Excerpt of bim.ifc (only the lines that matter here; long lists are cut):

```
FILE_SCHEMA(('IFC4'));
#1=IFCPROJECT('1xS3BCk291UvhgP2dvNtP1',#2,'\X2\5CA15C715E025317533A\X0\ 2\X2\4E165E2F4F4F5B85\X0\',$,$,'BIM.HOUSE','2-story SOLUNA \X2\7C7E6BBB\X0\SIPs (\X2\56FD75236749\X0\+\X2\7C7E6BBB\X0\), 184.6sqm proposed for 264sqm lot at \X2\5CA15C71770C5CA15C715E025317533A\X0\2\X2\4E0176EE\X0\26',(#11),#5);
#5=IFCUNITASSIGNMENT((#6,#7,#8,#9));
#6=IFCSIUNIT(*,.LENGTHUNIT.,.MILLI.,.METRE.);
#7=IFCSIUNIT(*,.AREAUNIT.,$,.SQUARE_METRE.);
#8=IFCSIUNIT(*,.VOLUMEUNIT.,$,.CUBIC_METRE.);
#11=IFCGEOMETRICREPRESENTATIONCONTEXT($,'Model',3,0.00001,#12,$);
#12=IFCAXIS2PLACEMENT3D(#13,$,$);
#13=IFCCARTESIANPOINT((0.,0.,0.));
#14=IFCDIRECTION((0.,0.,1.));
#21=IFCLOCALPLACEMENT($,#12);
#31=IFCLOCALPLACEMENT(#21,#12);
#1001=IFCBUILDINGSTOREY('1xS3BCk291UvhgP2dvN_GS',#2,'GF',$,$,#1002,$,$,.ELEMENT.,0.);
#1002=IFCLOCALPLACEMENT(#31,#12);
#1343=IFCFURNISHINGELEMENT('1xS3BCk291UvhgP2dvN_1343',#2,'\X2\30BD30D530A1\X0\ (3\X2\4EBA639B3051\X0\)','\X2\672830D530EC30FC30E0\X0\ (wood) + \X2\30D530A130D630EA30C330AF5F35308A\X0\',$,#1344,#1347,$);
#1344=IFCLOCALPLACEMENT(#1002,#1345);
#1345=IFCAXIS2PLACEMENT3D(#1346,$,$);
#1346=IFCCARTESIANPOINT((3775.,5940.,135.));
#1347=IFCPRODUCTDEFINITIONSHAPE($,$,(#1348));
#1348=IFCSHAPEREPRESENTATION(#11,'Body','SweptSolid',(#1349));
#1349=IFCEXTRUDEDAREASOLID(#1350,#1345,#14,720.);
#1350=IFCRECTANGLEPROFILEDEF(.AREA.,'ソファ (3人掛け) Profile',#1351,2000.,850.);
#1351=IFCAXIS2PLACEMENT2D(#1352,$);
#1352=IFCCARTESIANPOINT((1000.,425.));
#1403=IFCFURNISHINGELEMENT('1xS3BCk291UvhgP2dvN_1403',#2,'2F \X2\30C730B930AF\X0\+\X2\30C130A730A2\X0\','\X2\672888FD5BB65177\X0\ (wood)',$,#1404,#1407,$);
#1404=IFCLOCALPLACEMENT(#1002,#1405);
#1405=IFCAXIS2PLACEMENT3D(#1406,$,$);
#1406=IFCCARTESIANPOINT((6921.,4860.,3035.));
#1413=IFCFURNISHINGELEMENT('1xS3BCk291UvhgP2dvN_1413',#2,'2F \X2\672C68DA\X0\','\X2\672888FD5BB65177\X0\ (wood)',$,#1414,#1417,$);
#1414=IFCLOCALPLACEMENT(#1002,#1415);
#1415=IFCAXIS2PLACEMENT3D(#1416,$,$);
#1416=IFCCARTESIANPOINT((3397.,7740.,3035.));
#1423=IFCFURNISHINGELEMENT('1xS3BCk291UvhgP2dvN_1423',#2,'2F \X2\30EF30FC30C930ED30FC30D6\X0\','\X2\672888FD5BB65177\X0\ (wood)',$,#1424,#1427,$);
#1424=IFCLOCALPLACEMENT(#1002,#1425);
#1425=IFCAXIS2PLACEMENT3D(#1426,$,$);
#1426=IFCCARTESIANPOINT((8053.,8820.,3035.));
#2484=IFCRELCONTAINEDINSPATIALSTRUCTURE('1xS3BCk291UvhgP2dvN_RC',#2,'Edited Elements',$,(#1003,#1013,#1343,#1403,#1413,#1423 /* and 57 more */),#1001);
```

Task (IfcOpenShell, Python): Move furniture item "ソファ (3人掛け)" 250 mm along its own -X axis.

```python
import ifcopenshell
import ifcopenshell.api.geometry
import ifcopenshell.util.placement

model = ifcopenshell.open("bim.ifc")

item = model.by_id(1343)
matrix = ifcopenshell.util.placement.get_local_placement(item.ObjectPlacement)
matrix[:3, 3] -= matrix[:3, 0] * 250.0
ifcopenshell.api.geometry.edit_object_placement(model, product=item, matrix=matrix, is_si=False)

print(ifcopenshell.util.placement.get_local_placement(item.ObjectPlacement).round(3) + 0.0)

model.write("bim_edited.ifc")
```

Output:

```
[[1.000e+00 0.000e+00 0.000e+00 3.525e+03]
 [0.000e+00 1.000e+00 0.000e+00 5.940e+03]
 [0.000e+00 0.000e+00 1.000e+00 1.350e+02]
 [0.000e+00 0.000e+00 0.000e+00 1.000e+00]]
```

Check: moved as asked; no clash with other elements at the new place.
